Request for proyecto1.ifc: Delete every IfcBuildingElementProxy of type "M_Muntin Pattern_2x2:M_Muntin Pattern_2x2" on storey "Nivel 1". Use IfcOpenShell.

First a look at what the model holds.

```python
import ifcopenshell
import ifcopenshell.util.element

model = ifcopenshell.open("proyecto1.ifc")
print(model.schema)
storey = next(s for s in model.by_type("IfcBuildingStorey") if s.Name == "Nivel 1")
proxies = [e for e in ifcopenshell.util.element.get_decomposition(storey) if e.is_a("IfcBuildingElementProxy")]
seen = {}
for e in proxies:
    element_type = ifcopenshell.util.element.get_type(e)
    name = element_type.Name if element_type not in (None, e) else None
    seen[name] = seen.get(name, 0) + 1
for name, count in sorted(seen.items(), key=str):
    print(count, "x", name)
```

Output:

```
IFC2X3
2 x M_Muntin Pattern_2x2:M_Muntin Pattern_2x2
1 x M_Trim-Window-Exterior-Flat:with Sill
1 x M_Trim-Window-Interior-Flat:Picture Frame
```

```python
import ifcopenshell
import ifcopenshell.api.root
import ifcopenshell.util.element

model = ifcopenshell.open("proyecto1.ifc")

storey = next(s for s in model.by_type("IfcBuildingStorey") if s.Name == "Nivel 1")
proxies = [e for e in ifcopenshell.util.element.get_decomposition(storey) if e.is_a("IfcBuildingElementProxy")]
targets = [e for e in proxies if (t := ifcopenshell.util.element.get_type(e)) not in (None, e) and t.Name == "M_Muntin Pattern_2x2:M_Muntin Pattern_2x2"]

for e in targets:
    ifcopenshell.api.root.remove_product(model, product=e)
print(len(targets), "removed")

model.write("proyecto1_edited.ifc")
```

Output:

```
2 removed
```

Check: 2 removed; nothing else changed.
